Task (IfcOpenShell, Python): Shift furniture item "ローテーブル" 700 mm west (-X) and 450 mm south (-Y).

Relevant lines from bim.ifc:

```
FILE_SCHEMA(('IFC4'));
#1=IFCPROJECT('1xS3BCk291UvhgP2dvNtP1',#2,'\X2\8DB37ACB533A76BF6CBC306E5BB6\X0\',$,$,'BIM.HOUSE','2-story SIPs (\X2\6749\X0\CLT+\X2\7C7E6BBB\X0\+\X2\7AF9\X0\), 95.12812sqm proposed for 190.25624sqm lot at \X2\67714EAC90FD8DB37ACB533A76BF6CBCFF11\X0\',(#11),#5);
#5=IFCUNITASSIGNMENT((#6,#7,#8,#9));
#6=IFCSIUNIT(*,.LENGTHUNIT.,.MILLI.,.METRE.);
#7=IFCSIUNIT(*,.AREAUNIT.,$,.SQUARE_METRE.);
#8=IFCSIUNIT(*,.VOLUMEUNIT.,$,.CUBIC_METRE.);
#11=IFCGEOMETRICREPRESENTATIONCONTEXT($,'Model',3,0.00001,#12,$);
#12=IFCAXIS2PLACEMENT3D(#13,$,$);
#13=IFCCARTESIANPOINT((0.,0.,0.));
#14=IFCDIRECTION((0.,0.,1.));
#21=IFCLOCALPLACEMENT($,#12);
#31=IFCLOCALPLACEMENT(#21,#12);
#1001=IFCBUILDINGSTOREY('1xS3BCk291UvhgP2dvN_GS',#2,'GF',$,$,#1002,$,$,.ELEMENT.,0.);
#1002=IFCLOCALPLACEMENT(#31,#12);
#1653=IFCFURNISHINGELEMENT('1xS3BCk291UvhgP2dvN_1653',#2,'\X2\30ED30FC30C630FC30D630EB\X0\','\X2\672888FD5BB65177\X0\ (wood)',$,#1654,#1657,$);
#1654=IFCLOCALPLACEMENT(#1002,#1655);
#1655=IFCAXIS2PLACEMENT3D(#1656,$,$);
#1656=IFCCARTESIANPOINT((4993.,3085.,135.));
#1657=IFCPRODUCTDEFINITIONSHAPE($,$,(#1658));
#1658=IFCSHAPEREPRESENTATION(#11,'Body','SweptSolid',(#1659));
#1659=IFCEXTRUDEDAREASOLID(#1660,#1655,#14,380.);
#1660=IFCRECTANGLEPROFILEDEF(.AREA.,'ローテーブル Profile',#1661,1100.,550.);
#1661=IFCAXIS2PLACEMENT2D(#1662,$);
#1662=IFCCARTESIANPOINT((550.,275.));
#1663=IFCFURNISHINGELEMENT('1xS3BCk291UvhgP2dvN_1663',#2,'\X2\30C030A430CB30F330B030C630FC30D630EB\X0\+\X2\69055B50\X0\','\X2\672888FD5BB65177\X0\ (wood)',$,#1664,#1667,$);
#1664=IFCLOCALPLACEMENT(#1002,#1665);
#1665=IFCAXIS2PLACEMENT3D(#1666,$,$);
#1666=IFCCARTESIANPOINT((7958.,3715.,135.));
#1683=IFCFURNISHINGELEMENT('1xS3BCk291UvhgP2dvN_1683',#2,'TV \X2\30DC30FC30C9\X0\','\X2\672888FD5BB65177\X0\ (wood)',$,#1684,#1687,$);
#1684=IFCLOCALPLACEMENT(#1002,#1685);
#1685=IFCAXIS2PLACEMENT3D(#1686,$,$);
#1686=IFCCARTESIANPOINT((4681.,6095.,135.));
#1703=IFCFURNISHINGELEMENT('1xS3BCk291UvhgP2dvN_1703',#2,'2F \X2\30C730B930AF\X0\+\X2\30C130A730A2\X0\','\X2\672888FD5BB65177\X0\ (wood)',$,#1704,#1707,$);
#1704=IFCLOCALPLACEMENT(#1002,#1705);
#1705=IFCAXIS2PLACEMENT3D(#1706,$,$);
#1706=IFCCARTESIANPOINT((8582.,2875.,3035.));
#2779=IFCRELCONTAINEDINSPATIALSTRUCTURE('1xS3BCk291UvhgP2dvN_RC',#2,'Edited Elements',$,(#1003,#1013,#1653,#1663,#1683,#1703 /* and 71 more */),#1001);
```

```python
import ifcopenshell
import ifcopenshell.api.geometry
import ifcopenshell.util.placement
import ifcopenshell.util.unit

model = ifcopenshell.open("bim.ifc")
unit_scale = ifcopenshell.util.unit.calculate_unit_scale(model)

item = model.by_guid("1xS3BCk291UvhgP2dvN_1653")
matrix = ifcopenshell.util.placement.get_local_placement(item.ObjectPlacement)
matrix[0, 3] -= 0.7 / unit_scale
matrix[1, 3] -= 0.45 / unit_scale
ifcopenshell.api.geometry.edit_object_placement(model, product=item, matrix=matrix, is_si=False)

print(ifcopenshell.util.placement.get_local_placement(item.ObjectPlacement).round(3) + 0.0)

model.write("bim_rev.ifc")
```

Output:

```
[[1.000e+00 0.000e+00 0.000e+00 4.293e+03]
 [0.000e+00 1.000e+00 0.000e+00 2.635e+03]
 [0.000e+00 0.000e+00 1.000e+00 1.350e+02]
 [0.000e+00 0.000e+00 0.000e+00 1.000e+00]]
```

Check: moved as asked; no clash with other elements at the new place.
